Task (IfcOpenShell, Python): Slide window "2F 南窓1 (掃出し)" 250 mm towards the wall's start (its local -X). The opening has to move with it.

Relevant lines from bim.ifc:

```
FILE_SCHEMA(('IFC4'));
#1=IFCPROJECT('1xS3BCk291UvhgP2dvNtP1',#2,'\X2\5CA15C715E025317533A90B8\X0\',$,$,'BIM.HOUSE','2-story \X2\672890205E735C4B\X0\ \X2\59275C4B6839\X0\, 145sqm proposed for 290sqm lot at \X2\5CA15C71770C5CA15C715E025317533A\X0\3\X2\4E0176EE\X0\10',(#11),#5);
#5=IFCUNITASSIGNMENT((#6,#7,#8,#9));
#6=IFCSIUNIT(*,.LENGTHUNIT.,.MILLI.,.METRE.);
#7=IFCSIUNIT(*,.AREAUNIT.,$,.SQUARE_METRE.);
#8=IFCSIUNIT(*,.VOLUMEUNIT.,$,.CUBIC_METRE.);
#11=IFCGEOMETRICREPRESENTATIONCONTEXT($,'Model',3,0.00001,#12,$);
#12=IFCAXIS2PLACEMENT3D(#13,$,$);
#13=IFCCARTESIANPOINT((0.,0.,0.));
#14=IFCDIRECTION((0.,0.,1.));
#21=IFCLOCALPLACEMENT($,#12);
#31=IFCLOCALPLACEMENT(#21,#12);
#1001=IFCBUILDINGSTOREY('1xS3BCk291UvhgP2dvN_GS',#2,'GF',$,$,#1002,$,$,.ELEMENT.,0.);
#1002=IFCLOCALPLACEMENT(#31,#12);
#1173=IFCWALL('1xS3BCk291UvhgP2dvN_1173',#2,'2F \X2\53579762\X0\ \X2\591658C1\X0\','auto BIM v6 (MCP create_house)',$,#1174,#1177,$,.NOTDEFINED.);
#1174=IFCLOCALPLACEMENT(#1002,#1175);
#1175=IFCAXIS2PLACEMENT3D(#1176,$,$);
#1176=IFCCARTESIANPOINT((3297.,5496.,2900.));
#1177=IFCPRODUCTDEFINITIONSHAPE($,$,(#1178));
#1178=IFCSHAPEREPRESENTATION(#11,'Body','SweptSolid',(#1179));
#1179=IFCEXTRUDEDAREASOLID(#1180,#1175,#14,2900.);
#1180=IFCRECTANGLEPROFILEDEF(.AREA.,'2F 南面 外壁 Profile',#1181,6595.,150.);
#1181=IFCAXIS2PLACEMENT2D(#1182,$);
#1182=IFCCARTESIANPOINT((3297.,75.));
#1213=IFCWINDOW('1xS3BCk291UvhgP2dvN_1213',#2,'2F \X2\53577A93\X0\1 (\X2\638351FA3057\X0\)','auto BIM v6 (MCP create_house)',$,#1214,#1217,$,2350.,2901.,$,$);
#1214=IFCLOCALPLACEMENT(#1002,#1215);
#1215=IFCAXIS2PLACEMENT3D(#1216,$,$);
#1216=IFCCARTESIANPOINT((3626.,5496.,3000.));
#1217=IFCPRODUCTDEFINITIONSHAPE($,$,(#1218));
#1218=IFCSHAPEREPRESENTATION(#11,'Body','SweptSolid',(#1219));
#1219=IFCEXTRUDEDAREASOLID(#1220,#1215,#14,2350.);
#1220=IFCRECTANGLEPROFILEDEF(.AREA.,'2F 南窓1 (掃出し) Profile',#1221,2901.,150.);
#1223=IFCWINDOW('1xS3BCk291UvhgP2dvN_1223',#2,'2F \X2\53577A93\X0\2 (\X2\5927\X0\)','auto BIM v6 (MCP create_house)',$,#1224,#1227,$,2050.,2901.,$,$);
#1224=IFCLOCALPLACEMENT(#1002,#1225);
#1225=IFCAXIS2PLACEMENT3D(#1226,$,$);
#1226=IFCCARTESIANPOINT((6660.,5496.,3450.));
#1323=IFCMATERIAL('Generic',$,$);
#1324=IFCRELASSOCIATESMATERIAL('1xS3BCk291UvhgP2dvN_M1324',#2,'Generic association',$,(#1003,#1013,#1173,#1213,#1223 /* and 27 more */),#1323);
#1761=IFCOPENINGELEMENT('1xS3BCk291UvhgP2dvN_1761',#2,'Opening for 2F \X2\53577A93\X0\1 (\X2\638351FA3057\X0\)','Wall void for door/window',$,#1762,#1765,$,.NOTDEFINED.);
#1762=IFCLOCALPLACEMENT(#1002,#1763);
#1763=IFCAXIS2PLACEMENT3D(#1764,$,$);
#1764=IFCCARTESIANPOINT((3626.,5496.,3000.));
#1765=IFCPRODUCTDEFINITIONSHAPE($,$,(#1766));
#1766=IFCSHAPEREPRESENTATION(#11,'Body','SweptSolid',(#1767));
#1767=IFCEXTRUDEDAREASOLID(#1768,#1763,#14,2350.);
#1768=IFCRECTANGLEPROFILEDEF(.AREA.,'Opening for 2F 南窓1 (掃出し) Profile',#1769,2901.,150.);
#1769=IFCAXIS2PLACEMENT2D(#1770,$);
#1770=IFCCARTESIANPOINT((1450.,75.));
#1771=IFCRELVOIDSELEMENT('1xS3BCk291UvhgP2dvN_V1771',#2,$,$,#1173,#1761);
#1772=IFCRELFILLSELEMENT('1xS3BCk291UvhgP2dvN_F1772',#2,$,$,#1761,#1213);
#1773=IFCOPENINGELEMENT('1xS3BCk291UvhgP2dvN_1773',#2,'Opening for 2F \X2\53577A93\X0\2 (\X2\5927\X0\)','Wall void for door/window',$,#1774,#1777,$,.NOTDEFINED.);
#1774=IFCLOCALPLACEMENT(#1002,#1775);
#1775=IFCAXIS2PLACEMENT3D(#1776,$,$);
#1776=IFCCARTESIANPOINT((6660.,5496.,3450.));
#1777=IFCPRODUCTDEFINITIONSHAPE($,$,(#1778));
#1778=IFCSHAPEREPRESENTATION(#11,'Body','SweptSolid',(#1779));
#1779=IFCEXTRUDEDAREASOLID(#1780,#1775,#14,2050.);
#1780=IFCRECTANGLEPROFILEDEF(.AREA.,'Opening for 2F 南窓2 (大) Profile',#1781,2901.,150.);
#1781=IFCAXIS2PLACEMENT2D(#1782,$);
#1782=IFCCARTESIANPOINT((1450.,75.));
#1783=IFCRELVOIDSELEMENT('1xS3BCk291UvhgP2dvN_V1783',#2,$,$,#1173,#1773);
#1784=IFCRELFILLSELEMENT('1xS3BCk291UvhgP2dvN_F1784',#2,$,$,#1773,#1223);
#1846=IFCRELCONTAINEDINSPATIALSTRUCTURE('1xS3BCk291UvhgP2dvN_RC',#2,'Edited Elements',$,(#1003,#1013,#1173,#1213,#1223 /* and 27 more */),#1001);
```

```python
import ifcopenshell
import ifcopenshell.api.geometry
import ifcopenshell.util.placement

model = ifcopenshell.open("bim.ifc")

window = model.by_guid("1xS3BCk291UvhgP2dvN_1213")
opening = window.FillsVoids[0].RelatingOpeningElement
wall = opening.VoidsElements[0].RelatingBuildingElement

wall_matrix = ifcopenshell.util.placement.get_local_placement(wall.ObjectPlacement)
shift = wall_matrix[:3, 0] * -250.0
before = ifcopenshell.util.placement.get_local_placement(window.ObjectPlacement)[:3, 3].copy()

# The window is not placed relative to its opening, so move both.
for product in (opening, window):
    matrix = ifcopenshell.util.placement.get_local_placement(product.ObjectPlacement)
    matrix[:3, 3] += shift
    ifcopenshell.api.geometry.edit_object_placement(model, product=product, matrix=matrix, is_si=False)

after = ifcopenshell.util.placement.get_local_placement(window.ObjectPlacement)[:3, 3]
print("window moved by", (after - before).round(3) + 0.0)

model.write("bim_rev.ifc")
```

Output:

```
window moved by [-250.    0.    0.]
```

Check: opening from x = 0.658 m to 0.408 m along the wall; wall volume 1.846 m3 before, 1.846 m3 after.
